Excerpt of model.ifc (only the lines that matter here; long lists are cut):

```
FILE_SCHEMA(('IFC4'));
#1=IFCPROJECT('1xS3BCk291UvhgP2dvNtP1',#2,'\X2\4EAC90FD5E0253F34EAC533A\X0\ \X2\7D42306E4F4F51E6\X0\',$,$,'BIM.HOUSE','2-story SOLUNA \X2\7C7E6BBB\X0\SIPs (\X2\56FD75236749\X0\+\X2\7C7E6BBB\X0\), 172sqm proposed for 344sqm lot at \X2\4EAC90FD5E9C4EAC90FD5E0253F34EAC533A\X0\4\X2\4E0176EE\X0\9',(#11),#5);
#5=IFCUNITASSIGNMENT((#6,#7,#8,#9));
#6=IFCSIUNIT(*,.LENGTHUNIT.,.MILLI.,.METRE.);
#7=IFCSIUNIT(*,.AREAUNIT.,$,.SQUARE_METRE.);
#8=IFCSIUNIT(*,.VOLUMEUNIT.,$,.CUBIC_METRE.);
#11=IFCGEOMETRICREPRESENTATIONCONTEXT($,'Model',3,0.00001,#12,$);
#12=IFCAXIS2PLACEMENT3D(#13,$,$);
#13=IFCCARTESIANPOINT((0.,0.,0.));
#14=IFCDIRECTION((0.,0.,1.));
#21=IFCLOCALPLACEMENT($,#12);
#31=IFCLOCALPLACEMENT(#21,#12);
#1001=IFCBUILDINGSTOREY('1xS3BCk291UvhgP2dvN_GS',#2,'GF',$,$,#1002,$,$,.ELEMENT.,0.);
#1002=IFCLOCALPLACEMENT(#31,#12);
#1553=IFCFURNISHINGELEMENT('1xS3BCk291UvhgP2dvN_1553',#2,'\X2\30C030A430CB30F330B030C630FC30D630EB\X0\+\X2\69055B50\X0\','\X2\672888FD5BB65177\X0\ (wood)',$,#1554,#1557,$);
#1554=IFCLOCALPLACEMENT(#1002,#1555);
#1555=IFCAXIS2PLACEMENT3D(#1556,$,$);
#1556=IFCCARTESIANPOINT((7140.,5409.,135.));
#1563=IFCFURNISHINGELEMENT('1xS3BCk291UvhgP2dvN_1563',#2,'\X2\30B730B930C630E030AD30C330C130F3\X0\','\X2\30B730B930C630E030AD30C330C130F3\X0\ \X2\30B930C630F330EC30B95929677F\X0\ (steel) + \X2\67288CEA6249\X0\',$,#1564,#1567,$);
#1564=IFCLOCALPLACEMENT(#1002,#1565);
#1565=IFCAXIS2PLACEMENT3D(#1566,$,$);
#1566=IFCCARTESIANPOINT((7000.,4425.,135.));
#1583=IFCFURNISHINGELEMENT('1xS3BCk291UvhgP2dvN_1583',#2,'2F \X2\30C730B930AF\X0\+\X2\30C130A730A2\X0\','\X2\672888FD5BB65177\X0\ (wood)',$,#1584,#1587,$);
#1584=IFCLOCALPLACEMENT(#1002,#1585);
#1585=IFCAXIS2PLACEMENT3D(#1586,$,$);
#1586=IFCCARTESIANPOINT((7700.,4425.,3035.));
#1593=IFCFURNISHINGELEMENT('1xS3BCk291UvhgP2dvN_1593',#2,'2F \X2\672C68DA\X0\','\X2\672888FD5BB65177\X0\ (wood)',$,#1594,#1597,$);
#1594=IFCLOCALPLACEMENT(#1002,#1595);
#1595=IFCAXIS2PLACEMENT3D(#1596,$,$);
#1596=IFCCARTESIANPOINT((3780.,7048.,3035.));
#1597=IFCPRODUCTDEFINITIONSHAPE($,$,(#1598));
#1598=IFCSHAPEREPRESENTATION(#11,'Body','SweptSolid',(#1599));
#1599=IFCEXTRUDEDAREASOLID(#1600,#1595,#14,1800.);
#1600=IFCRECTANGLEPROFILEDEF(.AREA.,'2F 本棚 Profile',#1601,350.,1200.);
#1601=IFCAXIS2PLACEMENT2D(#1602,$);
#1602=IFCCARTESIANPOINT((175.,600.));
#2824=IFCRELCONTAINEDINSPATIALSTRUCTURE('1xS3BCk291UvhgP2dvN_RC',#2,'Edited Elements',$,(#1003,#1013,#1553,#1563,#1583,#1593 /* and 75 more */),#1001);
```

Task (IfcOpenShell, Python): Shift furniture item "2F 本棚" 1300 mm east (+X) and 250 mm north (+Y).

```python
import ifcopenshell
import ifcopenshell.api.geometry
import ifcopenshell.util.placement
import ifcopenshell.util.unit

model = ifcopenshell.open("model.ifc")
unit_scale = ifcopenshell.util.unit.calculate_unit_scale(model)

item = model.by_guid("1xS3BCk291UvhgP2dvN_1593")
matrix = ifcopenshell.util.placement.get_local_placement(item.ObjectPlacement)
matrix[0, 3] += 1.3 / unit_scale
matrix[1, 3] += 0.25 / unit_scale
ifcopenshell.api.geometry.edit_object_placement(model, product=item, matrix=matrix, is_si=False)

print(ifcopenshell.util.placement.get_local_placement(item.ObjectPlacement).round(3) + 0.0)

model.write("model_v2.ifc")
```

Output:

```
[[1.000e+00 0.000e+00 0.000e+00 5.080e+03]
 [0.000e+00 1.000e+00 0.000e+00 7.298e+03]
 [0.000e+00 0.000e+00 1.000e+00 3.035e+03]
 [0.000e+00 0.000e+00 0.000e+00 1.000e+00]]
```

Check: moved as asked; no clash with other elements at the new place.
